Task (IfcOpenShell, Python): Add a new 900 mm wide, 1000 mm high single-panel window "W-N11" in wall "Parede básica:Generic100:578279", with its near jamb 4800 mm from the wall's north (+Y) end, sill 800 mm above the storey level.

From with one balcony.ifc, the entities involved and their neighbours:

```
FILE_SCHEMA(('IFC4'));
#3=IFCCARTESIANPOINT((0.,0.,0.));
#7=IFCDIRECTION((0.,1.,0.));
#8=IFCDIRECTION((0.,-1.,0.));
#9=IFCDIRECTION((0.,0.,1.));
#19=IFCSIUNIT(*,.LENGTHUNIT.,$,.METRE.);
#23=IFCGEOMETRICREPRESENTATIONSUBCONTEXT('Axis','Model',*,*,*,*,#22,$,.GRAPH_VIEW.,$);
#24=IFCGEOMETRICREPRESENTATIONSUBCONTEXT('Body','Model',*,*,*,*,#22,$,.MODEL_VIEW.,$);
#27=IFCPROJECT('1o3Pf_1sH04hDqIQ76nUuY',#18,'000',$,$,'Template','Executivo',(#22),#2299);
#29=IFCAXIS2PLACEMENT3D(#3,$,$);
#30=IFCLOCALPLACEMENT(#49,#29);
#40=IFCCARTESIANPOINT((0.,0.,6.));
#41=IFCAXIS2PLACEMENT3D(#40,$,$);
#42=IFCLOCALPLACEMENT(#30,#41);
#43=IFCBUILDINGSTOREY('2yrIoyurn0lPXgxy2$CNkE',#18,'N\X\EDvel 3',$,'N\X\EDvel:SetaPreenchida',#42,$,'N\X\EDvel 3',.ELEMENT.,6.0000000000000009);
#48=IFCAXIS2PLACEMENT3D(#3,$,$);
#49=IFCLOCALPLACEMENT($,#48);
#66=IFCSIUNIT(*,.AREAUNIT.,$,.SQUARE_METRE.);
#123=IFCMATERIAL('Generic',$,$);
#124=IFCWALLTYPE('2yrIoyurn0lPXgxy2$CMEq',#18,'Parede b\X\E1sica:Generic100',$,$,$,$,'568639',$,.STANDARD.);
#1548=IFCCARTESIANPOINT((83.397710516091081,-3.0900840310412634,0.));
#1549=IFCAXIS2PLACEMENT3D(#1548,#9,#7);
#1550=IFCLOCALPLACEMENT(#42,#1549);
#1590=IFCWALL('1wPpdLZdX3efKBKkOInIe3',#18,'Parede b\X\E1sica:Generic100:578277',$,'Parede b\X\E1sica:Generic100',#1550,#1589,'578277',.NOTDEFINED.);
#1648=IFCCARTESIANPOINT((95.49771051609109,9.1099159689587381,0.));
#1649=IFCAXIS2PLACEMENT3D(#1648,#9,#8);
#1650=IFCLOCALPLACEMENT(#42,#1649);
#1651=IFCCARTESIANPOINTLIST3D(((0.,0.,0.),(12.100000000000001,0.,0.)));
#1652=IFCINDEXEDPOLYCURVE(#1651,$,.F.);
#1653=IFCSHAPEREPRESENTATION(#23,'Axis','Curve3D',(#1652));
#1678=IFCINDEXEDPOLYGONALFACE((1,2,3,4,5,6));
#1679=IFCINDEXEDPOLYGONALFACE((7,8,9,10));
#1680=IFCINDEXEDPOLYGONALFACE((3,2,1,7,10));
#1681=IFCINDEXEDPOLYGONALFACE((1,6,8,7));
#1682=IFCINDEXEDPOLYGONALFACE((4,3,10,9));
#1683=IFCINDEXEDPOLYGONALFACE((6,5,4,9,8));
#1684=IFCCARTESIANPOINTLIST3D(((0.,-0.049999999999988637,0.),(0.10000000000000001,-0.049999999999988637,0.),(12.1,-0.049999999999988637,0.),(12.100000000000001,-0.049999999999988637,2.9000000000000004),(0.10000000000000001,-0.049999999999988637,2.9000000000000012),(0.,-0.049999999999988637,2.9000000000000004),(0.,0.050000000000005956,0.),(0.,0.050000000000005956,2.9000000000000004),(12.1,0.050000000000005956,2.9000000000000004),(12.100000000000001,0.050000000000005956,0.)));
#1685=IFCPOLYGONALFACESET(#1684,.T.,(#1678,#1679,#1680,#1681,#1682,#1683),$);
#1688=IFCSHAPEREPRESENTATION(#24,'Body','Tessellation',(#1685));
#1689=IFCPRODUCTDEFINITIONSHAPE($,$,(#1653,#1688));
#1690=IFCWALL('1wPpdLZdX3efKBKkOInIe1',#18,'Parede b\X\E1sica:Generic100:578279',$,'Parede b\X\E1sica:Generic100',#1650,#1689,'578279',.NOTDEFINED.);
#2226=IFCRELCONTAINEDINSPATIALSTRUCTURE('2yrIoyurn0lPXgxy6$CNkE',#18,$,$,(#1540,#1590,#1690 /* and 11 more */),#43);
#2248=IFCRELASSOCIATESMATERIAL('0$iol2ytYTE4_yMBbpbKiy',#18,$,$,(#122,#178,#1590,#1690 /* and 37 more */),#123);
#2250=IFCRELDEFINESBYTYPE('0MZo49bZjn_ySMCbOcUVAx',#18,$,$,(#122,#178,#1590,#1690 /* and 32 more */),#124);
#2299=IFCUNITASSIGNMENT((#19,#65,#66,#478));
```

```python
import numpy as np
import ifcopenshell
import ifcopenshell.api.feature
import ifcopenshell.api.geometry
import ifcopenshell.api.root
import ifcopenshell.api.spatial
import ifcopenshell.geom
import ifcopenshell.util.element
import ifcopenshell.util.placement
import ifcopenshell.util.representation
import ifcopenshell.util.shape
import ifcopenshell.util.unit

model = ifcopenshell.open("with one balcony.ifc")
unit_scale = ifcopenshell.util.unit.calculate_unit_scale(model)
settings = ifcopenshell.geom.settings()


def volume(element):
    """Net volume in cubic metres, openings subtracted."""
    shape = ifcopenshell.geom.create_shape(settings, element)
    return ifcopenshell.util.shape.get_volume(shape.geometry)


wall = model.by_guid("1wPpdLZdX3efKBKkOInIe1")
storey = ifcopenshell.util.element.get_container(wall, ifc_class="IfcBuildingStorey")
context = ifcopenshell.util.representation.get_context(model, "Model", "Body", "MODEL_VIEW")
before = volume(wall)

width, height, from_end, sill = 0.9, 1, 4.8, 0.8  # metres

# The wall runs along its own X axis, and the end named is its -X end.
wall_shape = ifcopenshell.geom.create_shape(settings, wall)
x, y, z = ifcopenshell.util.shape.get_vertices(wall_shape.geometry).T
start = x.min() + from_end
face, thickness = float(y.min()), float(y.max() - y.min())
wall_matrix = ifcopenshell.util.placement.get_local_placement(wall.ObjectPlacement)
level = ifcopenshell.util.placement.get_local_placement(storey.ObjectPlacement)[2, 3]


def in_wall(x, y):
    """Placement at x, y metres in the wall's axes, at sill height."""
    matrix = wall_matrix.copy()
    matrix[:, 3] = wall_matrix @ np.array([x / unit_scale, y / unit_scale, 0.0, 1.0])
    matrix[2, 3] = level + sill / unit_scale
    return matrix


# Opening: a box that overshoots both wall faces by 50 mm.
opening = ifcopenshell.api.root.create_entity(model, ifc_class="IfcOpeningElement", predefined_type="OPENING")
box = ifcopenshell.api.geometry.add_wall_representation(
    model, context=context, length=width, height=height, thickness=thickness + 0.1
)
ifcopenshell.api.geometry.assign_representation(model, product=opening, representation=box)
ifcopenshell.api.geometry.edit_object_placement(model, product=opening, matrix=in_wall(start, face - 0.05), is_si=False)
ifcopenshell.api.feature.add_feature(model, feature=opening, element=wall)

window = ifcopenshell.api.root.create_entity(model, ifc_class="IfcWindow", name="W-N11", predefined_type="WINDOW")
window.OverallWidth, window.OverallHeight = width / unit_scale, height / unit_scale
window.PartitioningType = "SINGLE_PANEL"
body = ifcopenshell.api.geometry.add_window_representation(
    model,
    context=context,
    overall_width=window.OverallWidth,
    overall_height=window.OverallHeight,
    partition_type="SINGLE_PANEL",
)
ifcopenshell.api.geometry.assign_representation(model, product=window, representation=body)
ifcopenshell.api.spatial.assign_container(model, products=[window], relating_structure=storey)
ifcopenshell.api.feature.add_filling(model, opening=opening, element=window)

# Centre the window in the wall's thickness.
ifcopenshell.api.geometry.edit_object_placement(model, product=window, matrix=in_wall(start, face), is_si=False)
window_shape = ifcopenshell.geom.create_shape(settings, window)
depth = ifcopenshell.util.shape.get_vertices(window_shape.geometry)[:, 1]
offset = face + thickness / 2 - (depth.min() + depth.max()) / 2
ifcopenshell.api.geometry.edit_object_placement(model, product=window, matrix=in_wall(start, offset), is_si=False)

after = volume(wall)

print(f"wall volume {before:.3f} -> {after:.3f} m3")

model.write("with one balcony_updated.ifc")
```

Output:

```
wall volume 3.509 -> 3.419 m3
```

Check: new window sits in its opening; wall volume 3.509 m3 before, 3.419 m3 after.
